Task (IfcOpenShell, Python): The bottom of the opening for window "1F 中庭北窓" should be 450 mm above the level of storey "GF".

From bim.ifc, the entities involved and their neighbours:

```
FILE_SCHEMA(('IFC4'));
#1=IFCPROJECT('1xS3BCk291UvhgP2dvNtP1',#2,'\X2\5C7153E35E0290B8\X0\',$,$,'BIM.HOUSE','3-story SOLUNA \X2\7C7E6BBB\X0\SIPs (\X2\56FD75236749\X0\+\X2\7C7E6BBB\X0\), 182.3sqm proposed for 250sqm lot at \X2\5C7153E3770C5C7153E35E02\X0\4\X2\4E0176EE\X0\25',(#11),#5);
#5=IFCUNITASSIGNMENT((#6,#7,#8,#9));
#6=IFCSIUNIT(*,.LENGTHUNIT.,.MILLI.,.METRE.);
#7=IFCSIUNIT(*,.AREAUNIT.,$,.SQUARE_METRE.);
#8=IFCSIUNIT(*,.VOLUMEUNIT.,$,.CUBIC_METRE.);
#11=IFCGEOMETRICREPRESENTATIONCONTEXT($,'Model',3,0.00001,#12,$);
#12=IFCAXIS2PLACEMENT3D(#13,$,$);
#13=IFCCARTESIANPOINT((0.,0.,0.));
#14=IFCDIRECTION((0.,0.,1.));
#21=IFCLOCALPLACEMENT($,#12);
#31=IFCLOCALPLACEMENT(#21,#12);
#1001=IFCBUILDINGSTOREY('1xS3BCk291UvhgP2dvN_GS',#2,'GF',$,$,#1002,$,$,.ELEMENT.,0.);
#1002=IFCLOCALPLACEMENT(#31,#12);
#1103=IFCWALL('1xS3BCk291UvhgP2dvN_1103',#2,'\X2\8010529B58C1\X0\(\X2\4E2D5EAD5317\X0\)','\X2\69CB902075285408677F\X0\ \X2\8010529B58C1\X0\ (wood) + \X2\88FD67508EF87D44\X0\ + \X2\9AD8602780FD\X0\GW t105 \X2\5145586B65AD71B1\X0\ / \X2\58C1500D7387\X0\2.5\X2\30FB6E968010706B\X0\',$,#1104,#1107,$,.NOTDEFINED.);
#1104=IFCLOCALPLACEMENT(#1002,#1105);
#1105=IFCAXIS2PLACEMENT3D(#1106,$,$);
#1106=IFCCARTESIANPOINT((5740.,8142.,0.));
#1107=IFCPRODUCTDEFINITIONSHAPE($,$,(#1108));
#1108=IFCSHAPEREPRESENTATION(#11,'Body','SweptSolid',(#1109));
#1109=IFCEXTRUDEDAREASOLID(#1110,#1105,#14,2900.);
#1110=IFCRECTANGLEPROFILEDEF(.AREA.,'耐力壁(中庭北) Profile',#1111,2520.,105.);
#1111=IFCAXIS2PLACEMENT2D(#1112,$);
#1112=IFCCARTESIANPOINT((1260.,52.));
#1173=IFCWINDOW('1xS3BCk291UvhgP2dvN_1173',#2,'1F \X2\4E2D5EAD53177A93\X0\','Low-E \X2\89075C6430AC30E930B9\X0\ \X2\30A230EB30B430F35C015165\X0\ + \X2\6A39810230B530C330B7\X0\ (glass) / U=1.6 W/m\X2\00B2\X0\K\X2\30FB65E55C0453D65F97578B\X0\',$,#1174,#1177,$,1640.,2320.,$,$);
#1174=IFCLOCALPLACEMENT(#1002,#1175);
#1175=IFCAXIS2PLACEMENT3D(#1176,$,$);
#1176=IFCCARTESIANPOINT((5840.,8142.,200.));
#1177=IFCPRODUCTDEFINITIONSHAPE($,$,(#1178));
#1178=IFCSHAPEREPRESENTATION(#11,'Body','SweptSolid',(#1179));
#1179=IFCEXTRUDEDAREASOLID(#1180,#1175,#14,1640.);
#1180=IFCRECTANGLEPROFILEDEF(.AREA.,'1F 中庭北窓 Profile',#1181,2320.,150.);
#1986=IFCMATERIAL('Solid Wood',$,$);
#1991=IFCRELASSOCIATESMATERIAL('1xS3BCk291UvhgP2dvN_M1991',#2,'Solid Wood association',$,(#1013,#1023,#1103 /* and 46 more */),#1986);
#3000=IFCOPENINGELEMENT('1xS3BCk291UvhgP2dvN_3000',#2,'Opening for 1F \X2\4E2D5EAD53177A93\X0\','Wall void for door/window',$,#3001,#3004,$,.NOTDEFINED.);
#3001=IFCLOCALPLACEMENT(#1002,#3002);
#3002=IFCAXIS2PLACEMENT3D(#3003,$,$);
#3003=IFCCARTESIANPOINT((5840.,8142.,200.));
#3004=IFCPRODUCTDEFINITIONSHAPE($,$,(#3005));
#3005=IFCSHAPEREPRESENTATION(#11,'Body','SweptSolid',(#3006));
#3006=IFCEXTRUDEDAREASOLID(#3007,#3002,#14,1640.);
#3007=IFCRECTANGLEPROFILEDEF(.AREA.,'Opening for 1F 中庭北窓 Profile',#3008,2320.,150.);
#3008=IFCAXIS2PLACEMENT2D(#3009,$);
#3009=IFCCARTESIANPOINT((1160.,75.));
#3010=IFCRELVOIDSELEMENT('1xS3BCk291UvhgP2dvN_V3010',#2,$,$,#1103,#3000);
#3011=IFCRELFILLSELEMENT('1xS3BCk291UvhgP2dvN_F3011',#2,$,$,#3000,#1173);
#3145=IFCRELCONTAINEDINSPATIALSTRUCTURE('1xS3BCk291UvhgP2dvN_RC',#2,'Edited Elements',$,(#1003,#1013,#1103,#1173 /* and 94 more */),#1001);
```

```python
import numpy as np
import ifcopenshell
import ifcopenshell.api.geometry
import ifcopenshell.geom
import ifcopenshell.util.element
import ifcopenshell.util.placement
import ifcopenshell.util.shape
import ifcopenshell.util.unit

model = ifcopenshell.open("bim.ifc")
unit_scale = ifcopenshell.util.unit.calculate_unit_scale(model)

window = model.by_guid("1xS3BCk291UvhgP2dvN_1173")
opening = window.FillsVoids[0].RelatingOpeningElement
storey = ifcopenshell.util.element.get_container(window, ifc_class="IfcBuildingStorey")
level = ifcopenshell.util.placement.get_local_placement(storey.ObjectPlacement)[2, 3]

# The opening's origin need not be at the sill, so measure its lowest point.
shape = ifcopenshell.geom.create_shape(ifcopenshell.geom.settings(), opening)
bottom = ifcopenshell.util.shape.get_shape_bottom_elevation(shape, shape.geometry) / unit_scale
dz = level + 0.45 / unit_scale - bottom

shift = np.array([0.0, 0.0, dz])
# The window is not placed relative to its opening, so move both.
for product in (opening, window):
    matrix = ifcopenshell.util.placement.get_local_placement(product.ObjectPlacement)
    matrix[:3, 3] += shift
    ifcopenshell.api.geometry.edit_object_placement(model, product=product, matrix=matrix, is_si=False)

print(f"moved by {dz * unit_scale:+.3f} m")

model.write("bim_updated.ifc")
```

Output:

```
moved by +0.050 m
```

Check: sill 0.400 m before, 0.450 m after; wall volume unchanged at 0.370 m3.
